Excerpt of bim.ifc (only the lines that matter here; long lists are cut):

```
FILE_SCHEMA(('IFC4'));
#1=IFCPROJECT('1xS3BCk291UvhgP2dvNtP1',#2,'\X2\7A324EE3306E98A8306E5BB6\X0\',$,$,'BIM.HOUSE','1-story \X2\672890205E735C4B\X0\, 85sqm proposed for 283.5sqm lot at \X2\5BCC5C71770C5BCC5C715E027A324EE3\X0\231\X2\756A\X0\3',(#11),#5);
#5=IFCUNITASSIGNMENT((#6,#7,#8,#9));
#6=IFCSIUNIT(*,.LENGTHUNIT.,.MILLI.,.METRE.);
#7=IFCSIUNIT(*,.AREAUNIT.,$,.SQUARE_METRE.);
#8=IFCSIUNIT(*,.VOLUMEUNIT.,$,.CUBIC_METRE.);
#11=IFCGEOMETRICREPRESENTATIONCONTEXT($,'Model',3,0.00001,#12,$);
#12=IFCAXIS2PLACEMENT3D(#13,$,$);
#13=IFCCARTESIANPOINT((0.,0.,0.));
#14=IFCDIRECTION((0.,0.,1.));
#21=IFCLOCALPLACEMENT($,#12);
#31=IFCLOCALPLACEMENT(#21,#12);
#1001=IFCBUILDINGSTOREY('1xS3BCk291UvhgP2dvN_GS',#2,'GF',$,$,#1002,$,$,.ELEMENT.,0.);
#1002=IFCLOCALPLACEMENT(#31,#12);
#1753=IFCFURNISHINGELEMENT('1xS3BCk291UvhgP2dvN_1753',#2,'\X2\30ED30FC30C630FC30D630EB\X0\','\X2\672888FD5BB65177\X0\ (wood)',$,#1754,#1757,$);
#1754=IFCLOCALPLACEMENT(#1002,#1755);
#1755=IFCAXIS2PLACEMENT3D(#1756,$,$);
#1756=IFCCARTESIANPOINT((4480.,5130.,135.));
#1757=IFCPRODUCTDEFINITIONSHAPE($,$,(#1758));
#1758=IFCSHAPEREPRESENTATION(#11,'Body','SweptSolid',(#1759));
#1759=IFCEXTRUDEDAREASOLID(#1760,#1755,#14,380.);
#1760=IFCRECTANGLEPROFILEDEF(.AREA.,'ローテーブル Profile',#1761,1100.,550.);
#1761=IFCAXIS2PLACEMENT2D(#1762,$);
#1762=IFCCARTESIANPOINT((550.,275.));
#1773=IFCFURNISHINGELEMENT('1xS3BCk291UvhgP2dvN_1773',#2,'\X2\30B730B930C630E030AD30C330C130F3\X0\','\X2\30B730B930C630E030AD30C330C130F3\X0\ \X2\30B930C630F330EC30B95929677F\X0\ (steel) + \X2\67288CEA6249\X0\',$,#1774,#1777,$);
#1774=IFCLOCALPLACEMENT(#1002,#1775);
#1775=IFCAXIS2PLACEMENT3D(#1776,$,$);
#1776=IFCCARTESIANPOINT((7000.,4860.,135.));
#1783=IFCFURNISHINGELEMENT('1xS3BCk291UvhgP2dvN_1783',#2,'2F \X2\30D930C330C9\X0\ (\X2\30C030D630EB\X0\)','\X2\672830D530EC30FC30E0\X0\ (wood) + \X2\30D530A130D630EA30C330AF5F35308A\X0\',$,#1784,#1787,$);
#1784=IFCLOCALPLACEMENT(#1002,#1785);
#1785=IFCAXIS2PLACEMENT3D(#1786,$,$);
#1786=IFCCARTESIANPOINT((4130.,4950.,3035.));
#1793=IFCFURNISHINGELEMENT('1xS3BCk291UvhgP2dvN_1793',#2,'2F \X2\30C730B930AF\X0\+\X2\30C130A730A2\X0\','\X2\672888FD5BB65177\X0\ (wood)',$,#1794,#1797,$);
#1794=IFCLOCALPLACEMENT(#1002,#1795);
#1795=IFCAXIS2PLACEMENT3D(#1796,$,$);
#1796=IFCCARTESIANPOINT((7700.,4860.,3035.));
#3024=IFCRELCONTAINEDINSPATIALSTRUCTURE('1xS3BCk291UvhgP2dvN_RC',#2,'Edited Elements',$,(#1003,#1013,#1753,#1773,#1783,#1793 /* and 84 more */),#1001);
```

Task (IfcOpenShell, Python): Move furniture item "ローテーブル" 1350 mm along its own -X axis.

```python
import ifcopenshell
import ifcopenshell.api.geometry
import ifcopenshell.util.placement
import ifcopenshell.util.unit

model = ifcopenshell.open("bim.ifc")
unit_scale = ifcopenshell.util.unit.calculate_unit_scale(model)

item = model.by_guid("1xS3BCk291UvhgP2dvN_1753")
matrix = ifcopenshell.util.placement.get_local_placement(item.ObjectPlacement)
matrix[:3, 3] -= matrix[:3, 0] * 1.35 / unit_scale
ifcopenshell.api.geometry.edit_object_placement(model, product=item, matrix=matrix, is_si=False)

print(ifcopenshell.util.placement.get_local_placement(item.ObjectPlacement).round(3) + 0.0)

model.write("bim_edited.ifc")
```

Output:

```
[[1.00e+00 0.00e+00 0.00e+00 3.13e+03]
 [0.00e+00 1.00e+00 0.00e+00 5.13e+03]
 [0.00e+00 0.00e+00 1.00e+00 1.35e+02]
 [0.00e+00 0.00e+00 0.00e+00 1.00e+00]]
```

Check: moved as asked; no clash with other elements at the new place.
